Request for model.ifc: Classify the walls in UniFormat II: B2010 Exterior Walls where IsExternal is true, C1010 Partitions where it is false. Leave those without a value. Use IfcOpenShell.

First a look at what the model holds.

```python
import ifcopenshell
import ifcopenshell.util.element

model = ifcopenshell.open("model.ifc")
print(model.schema)
print("classifications:", [c.Name for c in model.by_type("IfcClassification")])
values = [ifcopenshell.util.element.get_pset(e, "Pset_WallCommon", "IsExternal") for e in model.by_type("IfcWall")]
for value in (True, False, None):
    print("IsExternal", value, values.count(value))
```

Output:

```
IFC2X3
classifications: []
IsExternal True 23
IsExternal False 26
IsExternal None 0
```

```python
import ifcopenshell
import ifcopenshell.api.classification
import ifcopenshell.util.element

model = ifcopenshell.open("model.ifc")

# IFC2X3 requires Source and Edition and has no link from the project to the system.
system = model.create_entity("IfcClassification", Source="ASTM", Edition="E1557", Name="UniFormat II")

walls = model.by_type("IfcWall")
external = {e: ifcopenshell.util.element.get_pset(e, "Pset_WallCommon", "IsExternal") for e in walls}
for flag, code, name in ((True, "B2010", "Exterior Walls"), (False, "C1010", "Partitions")):
    products = [e for e in walls if external[e] is flag]
    ifcopenshell.api.classification.add_reference(
        model, products=products, classification=system, identification=code, name=name
    )
    print(code, len(products))

model.write("model_edited.ifc")
```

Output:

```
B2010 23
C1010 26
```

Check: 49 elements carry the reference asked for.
